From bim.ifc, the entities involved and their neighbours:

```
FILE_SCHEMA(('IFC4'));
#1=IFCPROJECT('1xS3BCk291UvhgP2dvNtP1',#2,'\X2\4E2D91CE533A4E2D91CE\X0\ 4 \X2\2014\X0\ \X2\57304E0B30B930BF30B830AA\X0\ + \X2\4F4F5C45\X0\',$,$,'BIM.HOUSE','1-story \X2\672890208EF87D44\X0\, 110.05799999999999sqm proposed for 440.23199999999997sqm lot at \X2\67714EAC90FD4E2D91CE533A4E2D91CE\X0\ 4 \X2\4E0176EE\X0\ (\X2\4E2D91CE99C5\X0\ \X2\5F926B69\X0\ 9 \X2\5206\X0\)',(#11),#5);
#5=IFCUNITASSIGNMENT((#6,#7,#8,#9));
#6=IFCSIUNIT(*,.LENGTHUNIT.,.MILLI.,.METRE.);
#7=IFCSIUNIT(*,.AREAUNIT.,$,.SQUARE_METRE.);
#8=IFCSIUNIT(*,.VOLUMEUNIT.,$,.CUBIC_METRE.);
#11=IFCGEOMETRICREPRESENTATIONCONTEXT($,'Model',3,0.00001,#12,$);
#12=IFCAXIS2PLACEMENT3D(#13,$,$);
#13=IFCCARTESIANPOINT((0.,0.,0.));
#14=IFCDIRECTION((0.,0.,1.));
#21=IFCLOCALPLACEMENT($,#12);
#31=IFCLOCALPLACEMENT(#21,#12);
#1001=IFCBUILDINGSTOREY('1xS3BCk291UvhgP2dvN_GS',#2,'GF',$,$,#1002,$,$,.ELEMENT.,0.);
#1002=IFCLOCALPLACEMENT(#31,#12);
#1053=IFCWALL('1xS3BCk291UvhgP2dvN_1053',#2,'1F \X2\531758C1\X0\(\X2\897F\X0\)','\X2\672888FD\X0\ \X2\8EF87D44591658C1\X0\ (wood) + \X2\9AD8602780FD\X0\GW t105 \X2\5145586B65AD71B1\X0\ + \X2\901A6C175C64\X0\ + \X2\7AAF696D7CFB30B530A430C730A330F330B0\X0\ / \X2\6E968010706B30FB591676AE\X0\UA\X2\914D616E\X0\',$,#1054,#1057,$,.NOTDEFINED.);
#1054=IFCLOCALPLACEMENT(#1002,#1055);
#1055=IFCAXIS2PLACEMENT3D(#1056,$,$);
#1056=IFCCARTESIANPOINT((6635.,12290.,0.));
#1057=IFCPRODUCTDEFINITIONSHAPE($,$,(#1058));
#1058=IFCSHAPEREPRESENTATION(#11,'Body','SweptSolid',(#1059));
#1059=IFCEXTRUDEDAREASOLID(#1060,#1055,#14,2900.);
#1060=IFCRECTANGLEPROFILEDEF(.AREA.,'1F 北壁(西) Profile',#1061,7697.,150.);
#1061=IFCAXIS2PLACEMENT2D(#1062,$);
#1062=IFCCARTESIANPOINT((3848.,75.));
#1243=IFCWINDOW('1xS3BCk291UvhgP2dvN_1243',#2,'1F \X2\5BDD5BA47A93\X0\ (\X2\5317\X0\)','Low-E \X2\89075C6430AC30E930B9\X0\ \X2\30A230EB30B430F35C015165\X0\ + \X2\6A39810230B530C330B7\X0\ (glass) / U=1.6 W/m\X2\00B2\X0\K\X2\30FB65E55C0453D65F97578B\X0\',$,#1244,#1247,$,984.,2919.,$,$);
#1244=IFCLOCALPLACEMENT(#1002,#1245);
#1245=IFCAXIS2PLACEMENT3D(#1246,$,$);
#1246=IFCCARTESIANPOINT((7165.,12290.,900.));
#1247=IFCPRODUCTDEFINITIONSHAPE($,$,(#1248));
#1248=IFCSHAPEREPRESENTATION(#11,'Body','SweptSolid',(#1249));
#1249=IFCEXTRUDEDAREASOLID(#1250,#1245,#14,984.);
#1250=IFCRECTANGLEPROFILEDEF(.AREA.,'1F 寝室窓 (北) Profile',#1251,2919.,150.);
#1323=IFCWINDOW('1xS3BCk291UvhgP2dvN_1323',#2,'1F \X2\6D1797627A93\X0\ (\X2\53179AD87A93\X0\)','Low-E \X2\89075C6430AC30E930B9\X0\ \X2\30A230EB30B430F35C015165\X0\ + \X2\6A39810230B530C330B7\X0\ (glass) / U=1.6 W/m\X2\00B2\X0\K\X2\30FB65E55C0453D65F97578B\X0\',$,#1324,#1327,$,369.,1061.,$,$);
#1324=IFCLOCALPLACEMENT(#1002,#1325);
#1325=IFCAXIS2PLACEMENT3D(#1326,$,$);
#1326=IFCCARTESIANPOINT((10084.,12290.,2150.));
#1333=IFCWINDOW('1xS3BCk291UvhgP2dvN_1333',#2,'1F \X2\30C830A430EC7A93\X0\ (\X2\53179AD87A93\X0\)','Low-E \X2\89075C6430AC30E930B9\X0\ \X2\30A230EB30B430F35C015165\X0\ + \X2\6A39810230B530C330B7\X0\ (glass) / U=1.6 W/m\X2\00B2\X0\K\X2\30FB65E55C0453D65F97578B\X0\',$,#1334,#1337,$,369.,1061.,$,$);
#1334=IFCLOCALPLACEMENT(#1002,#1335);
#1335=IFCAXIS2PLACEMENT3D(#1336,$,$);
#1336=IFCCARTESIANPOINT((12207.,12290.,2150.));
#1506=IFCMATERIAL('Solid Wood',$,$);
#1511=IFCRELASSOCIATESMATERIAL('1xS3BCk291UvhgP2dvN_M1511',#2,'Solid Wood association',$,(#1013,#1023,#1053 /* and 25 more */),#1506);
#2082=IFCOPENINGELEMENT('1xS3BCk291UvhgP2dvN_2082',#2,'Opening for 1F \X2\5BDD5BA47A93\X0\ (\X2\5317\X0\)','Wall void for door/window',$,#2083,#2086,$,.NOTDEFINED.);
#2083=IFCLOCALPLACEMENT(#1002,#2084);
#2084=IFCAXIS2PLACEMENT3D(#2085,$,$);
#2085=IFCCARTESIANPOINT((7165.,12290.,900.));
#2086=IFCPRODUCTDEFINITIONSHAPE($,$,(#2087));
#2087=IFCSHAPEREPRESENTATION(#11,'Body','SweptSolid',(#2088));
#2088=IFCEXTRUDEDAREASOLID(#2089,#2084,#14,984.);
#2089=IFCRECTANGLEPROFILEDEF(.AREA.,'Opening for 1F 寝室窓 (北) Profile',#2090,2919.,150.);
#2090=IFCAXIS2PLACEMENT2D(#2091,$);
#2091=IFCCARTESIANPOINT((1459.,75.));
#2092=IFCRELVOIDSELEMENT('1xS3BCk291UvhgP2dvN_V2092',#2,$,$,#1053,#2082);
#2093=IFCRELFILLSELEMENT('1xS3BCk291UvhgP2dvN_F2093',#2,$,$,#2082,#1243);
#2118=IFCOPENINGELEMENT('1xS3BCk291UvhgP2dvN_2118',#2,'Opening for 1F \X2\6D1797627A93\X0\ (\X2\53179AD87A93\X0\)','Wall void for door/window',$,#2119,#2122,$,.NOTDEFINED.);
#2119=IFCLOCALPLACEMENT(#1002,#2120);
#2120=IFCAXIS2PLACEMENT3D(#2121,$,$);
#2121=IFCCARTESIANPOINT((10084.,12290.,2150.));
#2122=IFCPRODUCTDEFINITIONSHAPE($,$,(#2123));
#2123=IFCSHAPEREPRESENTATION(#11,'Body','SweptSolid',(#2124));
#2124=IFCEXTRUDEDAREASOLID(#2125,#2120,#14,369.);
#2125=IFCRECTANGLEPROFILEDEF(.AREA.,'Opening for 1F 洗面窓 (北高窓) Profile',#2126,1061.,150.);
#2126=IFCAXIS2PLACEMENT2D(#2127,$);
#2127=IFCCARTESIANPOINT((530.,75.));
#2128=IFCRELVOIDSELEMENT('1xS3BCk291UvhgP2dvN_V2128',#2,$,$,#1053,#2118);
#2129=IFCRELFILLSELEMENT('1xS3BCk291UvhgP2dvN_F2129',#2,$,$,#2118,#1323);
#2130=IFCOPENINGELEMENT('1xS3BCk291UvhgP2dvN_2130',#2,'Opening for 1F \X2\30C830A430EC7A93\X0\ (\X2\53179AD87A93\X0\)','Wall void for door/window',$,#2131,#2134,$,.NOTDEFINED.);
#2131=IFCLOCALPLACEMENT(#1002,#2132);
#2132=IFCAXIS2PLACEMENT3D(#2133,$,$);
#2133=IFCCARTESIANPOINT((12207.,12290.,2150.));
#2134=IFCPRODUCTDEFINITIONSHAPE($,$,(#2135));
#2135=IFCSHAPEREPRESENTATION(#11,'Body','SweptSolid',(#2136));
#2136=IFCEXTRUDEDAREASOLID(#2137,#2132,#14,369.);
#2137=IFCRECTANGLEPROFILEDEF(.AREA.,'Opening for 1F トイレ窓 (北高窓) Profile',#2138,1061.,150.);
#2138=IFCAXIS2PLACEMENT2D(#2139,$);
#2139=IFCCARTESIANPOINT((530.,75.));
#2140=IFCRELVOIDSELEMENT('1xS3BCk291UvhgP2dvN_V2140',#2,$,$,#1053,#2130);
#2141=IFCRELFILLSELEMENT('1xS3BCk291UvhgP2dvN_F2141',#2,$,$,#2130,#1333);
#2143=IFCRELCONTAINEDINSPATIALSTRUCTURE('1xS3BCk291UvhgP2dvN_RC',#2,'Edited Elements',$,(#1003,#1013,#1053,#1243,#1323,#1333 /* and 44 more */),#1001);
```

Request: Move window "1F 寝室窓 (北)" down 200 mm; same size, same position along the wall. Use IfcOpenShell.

```python
import numpy as np
import ifcopenshell
import ifcopenshell.api.geometry
import ifcopenshell.util.placement
import ifcopenshell.util.unit

model = ifcopenshell.open("bim.ifc")
unit_scale = ifcopenshell.util.unit.calculate_unit_scale(model)

window = model.by_guid("1xS3BCk291UvhgP2dvN_1243")
opening = window.FillsVoids[0].RelatingOpeningElement
dz = -200.0

shift = np.array([0.0, 0.0, dz])
# The window is not placed relative to its opening, so move both.
for product in (opening, window):
    matrix = ifcopenshell.util.placement.get_local_placement(product.ObjectPlacement)
    matrix[:3, 3] += shift
    ifcopenshell.api.geometry.edit_object_placement(model, product=product, matrix=matrix, is_si=False)

print(f"moved by {dz * unit_scale:+.3f} m")

model.write("bim_edited.ifc")
```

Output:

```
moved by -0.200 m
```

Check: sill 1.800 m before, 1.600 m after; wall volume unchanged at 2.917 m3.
